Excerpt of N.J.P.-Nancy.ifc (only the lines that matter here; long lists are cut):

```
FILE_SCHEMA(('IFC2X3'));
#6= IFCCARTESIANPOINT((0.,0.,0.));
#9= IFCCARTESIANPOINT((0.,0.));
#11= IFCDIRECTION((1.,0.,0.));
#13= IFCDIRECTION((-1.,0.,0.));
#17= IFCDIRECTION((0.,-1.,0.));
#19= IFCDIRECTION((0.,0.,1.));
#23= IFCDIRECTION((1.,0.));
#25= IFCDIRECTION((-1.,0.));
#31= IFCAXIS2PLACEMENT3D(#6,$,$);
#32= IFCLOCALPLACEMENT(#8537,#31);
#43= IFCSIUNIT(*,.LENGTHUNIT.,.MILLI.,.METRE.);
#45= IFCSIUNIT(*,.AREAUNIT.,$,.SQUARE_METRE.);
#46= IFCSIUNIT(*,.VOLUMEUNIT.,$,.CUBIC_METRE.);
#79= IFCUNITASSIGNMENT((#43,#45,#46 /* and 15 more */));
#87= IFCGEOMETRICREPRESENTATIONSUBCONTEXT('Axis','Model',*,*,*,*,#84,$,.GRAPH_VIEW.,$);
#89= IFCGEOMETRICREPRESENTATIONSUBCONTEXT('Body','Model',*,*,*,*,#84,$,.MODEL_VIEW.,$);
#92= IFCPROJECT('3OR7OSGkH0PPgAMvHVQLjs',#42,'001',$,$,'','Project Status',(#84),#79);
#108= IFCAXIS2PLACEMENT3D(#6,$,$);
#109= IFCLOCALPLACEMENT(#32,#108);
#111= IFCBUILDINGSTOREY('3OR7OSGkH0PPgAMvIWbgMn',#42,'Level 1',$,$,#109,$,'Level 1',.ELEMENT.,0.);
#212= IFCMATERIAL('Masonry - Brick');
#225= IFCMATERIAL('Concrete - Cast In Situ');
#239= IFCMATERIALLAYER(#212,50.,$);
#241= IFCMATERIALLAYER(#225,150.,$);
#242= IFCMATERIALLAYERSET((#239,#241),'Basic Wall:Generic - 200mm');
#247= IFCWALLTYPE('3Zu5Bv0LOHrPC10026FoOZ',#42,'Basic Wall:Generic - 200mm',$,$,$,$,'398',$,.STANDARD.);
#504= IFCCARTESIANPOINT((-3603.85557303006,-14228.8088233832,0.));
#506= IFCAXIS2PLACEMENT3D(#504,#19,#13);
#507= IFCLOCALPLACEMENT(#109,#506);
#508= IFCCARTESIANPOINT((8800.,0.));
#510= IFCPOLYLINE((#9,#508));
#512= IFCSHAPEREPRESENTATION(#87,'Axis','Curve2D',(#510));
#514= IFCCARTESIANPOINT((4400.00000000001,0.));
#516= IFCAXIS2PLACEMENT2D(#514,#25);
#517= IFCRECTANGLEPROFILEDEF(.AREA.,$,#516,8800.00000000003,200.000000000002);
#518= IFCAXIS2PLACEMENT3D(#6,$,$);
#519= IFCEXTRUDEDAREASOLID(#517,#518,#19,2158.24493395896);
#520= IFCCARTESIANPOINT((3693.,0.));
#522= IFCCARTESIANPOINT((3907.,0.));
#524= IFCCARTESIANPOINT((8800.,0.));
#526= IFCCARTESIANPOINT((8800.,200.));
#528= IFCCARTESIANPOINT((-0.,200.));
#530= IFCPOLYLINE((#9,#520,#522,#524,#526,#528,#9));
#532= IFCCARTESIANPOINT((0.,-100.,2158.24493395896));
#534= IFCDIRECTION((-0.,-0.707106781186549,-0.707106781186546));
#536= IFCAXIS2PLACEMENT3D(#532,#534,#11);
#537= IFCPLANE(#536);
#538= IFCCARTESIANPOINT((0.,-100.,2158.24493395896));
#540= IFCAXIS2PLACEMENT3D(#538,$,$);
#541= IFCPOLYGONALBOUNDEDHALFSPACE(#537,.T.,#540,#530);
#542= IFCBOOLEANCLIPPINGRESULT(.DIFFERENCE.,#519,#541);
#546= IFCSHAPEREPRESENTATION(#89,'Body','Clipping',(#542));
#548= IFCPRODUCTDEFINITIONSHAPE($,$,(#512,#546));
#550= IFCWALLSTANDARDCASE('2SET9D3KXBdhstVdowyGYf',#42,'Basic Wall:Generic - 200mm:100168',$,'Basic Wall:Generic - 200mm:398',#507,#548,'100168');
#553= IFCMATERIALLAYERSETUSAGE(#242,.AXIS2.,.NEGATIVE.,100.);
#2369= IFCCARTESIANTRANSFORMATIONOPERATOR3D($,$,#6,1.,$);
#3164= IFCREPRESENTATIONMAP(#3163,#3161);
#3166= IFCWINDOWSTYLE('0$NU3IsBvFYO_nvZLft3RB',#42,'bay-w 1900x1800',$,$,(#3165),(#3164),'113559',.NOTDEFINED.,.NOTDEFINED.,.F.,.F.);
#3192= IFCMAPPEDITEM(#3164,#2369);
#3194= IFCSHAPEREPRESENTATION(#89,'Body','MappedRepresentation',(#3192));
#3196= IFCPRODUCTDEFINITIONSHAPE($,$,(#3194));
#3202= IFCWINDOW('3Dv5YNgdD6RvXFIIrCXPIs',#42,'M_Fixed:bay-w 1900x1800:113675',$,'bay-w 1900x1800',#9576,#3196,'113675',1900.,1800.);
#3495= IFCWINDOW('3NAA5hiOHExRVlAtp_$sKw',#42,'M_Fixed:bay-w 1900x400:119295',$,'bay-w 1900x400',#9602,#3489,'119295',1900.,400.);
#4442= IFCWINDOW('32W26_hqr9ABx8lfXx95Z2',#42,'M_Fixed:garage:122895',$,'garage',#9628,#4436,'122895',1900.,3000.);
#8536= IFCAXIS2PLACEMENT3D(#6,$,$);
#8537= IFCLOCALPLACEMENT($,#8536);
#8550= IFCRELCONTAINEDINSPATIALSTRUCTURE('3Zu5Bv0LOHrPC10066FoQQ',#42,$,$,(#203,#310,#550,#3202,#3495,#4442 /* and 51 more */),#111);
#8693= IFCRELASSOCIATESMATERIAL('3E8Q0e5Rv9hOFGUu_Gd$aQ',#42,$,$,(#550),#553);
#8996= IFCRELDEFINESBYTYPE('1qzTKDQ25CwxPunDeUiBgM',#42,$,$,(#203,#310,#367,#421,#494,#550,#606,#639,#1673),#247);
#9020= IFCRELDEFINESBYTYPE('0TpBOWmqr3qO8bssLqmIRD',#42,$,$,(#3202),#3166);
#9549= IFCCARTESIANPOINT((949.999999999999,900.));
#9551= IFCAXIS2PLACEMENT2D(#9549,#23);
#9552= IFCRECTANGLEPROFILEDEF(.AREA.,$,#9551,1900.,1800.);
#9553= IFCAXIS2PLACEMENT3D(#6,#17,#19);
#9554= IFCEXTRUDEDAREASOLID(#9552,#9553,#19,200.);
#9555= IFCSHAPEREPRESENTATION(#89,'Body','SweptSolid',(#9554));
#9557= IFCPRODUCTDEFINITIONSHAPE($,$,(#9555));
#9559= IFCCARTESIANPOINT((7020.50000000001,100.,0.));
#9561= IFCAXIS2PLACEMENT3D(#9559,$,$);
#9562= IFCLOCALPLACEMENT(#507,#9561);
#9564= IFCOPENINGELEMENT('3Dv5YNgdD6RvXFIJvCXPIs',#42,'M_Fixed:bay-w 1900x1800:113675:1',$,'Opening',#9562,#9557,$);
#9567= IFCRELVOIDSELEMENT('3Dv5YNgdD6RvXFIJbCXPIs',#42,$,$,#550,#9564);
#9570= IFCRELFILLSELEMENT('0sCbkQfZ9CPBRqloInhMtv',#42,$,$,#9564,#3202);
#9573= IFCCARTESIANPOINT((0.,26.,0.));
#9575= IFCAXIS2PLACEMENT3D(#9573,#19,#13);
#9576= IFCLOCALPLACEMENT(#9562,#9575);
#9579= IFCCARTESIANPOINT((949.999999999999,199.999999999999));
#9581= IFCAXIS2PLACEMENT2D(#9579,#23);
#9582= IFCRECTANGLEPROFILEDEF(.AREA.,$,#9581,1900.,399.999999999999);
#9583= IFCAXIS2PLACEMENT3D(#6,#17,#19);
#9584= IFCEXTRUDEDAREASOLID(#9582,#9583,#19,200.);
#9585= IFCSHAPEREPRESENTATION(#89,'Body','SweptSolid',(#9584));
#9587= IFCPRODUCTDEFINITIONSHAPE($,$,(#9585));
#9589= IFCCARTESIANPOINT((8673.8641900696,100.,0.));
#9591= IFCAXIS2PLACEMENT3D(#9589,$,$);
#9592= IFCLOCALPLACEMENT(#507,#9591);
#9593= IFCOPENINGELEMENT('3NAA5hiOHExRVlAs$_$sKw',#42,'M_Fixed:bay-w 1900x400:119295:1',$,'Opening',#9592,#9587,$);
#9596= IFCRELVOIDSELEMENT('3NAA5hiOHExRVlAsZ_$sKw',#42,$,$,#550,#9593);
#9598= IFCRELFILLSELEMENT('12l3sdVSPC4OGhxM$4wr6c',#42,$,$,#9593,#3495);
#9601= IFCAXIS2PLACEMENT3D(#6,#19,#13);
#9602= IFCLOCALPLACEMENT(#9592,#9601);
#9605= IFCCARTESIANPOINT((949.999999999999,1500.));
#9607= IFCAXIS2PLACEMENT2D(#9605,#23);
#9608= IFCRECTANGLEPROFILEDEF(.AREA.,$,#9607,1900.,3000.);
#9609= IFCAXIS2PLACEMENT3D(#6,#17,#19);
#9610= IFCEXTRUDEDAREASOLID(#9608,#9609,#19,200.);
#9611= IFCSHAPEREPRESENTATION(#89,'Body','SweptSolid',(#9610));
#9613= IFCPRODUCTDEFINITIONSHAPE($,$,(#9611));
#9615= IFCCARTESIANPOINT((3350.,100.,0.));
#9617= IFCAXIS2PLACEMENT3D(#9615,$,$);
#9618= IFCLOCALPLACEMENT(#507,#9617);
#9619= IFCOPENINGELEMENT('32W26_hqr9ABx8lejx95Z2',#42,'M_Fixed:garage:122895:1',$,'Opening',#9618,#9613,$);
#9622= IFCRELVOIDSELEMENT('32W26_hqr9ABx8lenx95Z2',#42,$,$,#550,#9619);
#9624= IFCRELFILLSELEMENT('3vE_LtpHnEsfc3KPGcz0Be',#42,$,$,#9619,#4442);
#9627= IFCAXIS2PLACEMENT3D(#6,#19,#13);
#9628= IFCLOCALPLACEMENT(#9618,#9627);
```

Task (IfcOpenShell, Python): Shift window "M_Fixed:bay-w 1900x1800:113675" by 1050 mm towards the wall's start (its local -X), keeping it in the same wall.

```python
import ifcopenshell
import ifcopenshell.api.geometry
import ifcopenshell.util.placement

model = ifcopenshell.open("N.J.P.-Nancy.ifc")

window = model.by_id(3202)
opening = window.FillsVoids[0].RelatingOpeningElement
wall = opening.VoidsElements[0].RelatingBuildingElement

wall_matrix = ifcopenshell.util.placement.get_local_placement(wall.ObjectPlacement)
shift = wall_matrix[:3, 0] * -1050.0
before = ifcopenshell.util.placement.get_local_placement(window.ObjectPlacement)[:3, 3].copy()

# The window is placed relative to its opening, so it follows when the opening moves.
matrix = ifcopenshell.util.placement.get_local_placement(opening.ObjectPlacement)
matrix[:3, 3] += shift
ifcopenshell.api.geometry.edit_object_placement(
    model, product=opening, matrix=matrix, is_si=False, should_transform_children=True
)

after = ifcopenshell.util.placement.get_local_placement(window.ObjectPlacement)[:3, 3]
print("window moved by", (after - before).round(3) + 0.0)

model.write("N.J.P.-Nancy_rev.ifc")
```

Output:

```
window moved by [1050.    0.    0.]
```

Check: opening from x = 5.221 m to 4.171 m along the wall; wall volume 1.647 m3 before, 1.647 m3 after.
